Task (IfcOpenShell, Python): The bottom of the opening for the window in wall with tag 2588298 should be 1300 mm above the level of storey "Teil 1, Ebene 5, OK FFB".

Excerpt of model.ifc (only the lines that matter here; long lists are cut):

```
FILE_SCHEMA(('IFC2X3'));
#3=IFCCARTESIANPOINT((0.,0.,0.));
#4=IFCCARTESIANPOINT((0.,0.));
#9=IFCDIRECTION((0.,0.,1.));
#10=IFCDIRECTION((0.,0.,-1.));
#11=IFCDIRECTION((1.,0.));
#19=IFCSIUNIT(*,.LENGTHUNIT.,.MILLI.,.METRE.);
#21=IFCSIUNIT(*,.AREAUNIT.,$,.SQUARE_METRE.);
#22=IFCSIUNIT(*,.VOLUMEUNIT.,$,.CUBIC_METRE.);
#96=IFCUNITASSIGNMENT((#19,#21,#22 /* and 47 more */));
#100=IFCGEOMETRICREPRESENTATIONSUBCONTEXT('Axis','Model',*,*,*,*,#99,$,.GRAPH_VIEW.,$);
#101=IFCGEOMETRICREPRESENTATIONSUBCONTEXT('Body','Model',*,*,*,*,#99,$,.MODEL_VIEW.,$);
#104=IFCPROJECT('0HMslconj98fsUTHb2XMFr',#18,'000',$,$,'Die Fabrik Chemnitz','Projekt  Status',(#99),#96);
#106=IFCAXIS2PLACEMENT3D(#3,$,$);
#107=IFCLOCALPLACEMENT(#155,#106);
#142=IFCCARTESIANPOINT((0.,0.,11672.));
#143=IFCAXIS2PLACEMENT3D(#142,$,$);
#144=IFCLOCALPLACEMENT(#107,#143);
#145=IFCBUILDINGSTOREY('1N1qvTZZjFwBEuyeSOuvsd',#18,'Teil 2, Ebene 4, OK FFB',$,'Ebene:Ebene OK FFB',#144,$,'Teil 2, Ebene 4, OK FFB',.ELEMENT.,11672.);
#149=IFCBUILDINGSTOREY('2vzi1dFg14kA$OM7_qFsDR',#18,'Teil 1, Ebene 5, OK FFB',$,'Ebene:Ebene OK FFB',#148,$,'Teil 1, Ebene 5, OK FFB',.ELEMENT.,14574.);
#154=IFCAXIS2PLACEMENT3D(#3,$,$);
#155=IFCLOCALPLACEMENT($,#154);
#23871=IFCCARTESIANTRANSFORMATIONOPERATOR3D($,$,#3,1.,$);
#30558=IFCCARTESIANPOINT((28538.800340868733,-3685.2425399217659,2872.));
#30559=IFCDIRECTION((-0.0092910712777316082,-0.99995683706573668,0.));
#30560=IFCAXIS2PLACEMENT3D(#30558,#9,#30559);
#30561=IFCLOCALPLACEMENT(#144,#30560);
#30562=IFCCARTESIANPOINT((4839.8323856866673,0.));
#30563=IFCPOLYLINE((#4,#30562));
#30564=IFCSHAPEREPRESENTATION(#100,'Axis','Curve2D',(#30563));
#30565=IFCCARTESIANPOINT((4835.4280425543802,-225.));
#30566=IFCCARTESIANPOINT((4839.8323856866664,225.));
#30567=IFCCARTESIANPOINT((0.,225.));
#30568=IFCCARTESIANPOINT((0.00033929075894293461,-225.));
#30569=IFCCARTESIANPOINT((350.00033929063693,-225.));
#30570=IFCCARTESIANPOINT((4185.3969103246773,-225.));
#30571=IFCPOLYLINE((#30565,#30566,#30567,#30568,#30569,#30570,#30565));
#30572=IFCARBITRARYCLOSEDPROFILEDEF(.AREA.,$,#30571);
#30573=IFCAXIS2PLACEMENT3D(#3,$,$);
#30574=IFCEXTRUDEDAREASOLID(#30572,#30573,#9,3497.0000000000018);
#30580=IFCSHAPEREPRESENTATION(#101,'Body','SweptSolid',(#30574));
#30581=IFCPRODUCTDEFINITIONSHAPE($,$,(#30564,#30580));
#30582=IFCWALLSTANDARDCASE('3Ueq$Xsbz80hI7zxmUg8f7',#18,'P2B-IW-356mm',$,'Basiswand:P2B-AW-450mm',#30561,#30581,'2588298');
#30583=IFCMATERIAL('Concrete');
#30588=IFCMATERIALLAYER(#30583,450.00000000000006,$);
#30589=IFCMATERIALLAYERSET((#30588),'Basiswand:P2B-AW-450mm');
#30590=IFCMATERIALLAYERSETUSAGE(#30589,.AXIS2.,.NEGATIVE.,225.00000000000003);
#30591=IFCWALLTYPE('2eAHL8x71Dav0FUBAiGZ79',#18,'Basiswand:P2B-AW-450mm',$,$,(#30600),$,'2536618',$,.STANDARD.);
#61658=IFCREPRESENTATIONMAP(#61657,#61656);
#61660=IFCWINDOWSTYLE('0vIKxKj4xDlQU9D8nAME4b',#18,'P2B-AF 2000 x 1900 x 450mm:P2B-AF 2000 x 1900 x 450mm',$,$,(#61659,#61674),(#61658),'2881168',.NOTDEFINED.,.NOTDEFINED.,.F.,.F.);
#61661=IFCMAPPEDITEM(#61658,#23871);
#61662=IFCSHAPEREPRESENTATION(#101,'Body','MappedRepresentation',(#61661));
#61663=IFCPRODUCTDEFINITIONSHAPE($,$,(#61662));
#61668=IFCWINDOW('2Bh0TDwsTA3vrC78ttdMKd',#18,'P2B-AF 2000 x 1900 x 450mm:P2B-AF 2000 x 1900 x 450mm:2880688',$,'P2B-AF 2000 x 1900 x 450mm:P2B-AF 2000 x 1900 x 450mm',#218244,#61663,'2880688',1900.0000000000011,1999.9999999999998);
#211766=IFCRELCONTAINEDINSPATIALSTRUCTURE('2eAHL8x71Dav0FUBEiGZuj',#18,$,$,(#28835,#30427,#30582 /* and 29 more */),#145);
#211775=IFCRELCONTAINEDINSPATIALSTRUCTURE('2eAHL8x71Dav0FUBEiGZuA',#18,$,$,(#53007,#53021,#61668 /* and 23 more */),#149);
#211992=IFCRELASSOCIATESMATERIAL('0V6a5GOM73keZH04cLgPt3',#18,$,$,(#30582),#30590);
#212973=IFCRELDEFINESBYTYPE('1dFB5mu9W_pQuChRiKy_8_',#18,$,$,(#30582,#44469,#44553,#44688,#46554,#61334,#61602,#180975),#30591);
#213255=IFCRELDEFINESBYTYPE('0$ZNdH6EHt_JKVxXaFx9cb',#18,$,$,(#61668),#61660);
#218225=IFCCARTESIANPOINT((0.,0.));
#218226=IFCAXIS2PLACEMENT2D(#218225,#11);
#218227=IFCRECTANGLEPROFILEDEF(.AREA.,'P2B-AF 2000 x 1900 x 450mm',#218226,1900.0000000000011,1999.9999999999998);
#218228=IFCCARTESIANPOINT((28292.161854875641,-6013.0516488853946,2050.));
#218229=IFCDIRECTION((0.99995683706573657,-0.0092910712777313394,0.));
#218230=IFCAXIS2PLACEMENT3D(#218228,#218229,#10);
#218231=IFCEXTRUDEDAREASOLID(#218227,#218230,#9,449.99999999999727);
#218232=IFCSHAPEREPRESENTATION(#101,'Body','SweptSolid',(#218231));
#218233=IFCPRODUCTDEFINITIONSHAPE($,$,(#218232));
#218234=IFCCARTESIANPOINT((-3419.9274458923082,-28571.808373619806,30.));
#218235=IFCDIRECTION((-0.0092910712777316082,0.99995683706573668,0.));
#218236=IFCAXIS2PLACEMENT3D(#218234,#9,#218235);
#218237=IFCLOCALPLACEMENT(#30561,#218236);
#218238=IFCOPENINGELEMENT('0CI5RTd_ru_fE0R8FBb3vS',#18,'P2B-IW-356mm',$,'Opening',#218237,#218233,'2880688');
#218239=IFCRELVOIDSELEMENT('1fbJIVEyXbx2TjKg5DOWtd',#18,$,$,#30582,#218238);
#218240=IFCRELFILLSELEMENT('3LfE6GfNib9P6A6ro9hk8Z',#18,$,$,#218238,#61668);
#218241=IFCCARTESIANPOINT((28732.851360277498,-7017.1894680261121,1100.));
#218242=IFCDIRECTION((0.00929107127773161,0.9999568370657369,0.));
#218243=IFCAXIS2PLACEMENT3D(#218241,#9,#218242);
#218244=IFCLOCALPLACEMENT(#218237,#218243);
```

```python
import numpy as np
import ifcopenshell
import ifcopenshell.api.geometry
import ifcopenshell.geom
import ifcopenshell.util.element
import ifcopenshell.util.placement
import ifcopenshell.util.shape
import ifcopenshell.util.unit

model = ifcopenshell.open("model.ifc")
unit_scale = ifcopenshell.util.unit.calculate_unit_scale(model)

window = model.by_id(61668)
opening = window.FillsVoids[0].RelatingOpeningElement
storey = ifcopenshell.util.element.get_container(window, ifc_class="IfcBuildingStorey")
level = ifcopenshell.util.placement.get_local_placement(storey.ObjectPlacement)[2, 3]

# The opening's origin need not be at the sill, so measure its lowest point.
shape = ifcopenshell.geom.create_shape(ifcopenshell.geom.settings(), opening)
bottom = ifcopenshell.util.shape.get_shape_bottom_elevation(shape, shape.geometry) / unit_scale
dz = level + 1.3 / unit_scale - bottom

shift = np.array([0.0, 0.0, dz])
# The window is placed relative to its opening, so it follows when the opening moves.
matrix = ifcopenshell.util.placement.get_local_placement(opening.ObjectPlacement)
matrix[:3, 3] += shift
ifcopenshell.api.geometry.edit_object_placement(
    model, product=opening, matrix=matrix, is_si=False, should_transform_children=True
)

print(f"moved by {dz * unit_scale:+.3f} m")

model.write("model_edited.ifc")
```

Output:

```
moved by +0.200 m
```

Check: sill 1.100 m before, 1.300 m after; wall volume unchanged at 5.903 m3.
